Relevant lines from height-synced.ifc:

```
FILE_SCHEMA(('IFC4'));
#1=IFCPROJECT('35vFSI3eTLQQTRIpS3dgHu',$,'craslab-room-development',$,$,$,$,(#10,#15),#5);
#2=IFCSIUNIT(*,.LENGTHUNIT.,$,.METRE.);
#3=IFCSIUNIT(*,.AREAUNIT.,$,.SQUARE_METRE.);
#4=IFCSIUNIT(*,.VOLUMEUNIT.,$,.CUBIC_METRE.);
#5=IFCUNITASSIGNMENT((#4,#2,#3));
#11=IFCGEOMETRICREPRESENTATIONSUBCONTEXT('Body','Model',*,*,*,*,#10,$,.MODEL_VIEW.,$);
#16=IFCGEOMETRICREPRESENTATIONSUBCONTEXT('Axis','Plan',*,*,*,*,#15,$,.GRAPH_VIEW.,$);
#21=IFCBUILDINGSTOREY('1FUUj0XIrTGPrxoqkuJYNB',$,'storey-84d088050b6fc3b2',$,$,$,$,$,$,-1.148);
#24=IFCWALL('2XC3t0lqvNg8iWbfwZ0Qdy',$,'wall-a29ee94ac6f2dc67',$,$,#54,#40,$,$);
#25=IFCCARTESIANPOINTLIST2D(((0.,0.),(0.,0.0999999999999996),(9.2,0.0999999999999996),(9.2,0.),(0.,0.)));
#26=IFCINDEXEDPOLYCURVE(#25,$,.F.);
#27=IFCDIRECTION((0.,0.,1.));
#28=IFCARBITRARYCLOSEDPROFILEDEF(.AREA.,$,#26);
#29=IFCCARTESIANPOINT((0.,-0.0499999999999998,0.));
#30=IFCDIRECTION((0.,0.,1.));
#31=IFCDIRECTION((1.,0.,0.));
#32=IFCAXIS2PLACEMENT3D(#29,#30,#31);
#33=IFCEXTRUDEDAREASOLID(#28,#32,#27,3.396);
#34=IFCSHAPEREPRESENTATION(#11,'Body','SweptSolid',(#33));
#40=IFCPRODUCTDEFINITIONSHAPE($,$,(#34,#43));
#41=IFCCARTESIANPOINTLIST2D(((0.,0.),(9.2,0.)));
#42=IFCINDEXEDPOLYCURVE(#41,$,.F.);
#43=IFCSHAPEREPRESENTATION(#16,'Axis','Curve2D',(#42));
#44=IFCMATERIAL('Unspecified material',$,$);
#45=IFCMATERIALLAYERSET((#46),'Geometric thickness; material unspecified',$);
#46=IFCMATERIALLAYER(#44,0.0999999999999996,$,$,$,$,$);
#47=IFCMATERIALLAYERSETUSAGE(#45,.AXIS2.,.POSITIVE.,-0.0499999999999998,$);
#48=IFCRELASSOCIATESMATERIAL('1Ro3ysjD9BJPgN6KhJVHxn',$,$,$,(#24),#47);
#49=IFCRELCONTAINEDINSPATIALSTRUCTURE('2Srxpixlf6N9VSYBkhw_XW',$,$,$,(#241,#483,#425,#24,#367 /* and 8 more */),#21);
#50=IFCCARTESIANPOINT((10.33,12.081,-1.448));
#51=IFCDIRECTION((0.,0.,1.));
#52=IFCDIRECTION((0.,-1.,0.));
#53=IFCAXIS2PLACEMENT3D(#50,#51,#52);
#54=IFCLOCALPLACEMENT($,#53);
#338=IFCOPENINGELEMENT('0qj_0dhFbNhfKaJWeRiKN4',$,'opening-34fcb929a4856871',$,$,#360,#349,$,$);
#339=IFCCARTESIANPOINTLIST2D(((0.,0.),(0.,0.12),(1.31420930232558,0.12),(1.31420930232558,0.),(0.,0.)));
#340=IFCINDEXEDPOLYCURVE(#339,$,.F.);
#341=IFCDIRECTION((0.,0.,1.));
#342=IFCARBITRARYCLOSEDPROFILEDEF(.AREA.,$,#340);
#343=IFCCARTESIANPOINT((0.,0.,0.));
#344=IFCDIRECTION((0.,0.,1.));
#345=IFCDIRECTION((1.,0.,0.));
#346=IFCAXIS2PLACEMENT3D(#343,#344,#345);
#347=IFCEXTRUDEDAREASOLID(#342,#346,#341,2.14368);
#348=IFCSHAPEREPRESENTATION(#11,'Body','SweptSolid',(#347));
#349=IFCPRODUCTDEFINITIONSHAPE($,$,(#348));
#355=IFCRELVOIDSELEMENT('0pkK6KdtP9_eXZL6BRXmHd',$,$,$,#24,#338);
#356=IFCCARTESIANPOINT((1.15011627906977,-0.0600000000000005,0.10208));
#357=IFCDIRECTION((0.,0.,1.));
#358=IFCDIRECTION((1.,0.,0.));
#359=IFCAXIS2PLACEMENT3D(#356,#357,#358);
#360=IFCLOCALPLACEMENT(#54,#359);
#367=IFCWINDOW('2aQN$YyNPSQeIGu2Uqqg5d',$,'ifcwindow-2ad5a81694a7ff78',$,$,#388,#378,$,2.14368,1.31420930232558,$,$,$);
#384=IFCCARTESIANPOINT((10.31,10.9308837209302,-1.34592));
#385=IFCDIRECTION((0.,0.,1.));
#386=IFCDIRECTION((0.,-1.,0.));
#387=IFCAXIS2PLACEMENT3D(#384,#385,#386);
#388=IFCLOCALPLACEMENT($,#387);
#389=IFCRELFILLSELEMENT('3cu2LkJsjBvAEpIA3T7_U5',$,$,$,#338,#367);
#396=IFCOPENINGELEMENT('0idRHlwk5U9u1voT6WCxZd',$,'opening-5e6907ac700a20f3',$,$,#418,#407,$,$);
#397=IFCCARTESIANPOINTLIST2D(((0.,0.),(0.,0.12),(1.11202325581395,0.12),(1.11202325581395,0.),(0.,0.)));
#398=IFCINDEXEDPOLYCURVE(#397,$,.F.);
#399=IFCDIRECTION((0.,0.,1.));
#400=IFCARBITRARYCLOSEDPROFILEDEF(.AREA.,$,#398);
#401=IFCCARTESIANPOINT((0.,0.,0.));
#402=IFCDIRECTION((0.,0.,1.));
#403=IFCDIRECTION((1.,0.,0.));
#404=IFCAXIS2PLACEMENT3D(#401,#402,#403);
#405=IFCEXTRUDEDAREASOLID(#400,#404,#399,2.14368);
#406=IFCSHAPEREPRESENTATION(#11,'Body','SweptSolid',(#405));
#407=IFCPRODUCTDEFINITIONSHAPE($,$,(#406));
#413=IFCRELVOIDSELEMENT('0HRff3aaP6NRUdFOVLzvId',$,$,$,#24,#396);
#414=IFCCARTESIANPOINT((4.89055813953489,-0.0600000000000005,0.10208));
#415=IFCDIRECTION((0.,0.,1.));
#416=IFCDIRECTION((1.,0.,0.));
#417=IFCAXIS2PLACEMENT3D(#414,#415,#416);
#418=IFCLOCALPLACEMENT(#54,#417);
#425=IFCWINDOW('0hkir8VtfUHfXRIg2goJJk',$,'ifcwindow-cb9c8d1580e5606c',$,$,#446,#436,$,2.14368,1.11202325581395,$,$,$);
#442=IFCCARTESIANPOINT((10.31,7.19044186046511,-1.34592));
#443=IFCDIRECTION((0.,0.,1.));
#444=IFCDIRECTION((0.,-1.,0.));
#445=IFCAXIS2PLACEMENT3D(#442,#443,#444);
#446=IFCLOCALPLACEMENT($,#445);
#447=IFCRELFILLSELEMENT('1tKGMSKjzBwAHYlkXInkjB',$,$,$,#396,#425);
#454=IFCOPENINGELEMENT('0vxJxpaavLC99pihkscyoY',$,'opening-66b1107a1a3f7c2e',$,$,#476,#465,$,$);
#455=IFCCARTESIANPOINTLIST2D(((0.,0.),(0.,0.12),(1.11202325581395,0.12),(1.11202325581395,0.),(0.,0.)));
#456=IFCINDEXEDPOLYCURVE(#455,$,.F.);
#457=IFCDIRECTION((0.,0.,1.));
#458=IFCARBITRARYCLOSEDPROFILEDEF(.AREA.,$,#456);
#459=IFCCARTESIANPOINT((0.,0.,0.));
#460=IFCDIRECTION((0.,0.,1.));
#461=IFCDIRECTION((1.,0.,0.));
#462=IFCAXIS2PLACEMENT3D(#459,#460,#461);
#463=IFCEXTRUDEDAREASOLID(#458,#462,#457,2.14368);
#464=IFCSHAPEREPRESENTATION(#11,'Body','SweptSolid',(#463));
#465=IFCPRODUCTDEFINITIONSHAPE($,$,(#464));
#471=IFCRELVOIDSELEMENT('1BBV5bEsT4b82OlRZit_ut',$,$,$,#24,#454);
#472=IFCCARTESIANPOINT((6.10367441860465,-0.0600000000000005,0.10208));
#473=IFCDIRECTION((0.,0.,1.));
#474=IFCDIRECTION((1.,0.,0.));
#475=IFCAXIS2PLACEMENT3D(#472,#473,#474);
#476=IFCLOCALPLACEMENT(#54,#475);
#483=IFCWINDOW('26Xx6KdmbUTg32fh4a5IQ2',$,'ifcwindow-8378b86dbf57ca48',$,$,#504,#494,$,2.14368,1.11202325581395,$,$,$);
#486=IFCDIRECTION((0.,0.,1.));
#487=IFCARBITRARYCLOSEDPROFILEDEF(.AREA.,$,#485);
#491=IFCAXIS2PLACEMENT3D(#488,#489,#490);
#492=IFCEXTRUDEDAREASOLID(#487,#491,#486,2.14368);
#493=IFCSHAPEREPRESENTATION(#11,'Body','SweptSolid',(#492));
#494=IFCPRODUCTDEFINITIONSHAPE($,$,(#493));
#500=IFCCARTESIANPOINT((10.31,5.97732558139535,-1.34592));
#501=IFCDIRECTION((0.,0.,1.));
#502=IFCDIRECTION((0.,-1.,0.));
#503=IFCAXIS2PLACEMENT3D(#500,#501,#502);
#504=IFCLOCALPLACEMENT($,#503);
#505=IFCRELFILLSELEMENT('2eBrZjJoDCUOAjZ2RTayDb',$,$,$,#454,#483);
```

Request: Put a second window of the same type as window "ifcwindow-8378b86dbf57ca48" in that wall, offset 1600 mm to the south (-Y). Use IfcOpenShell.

```python
import ifcopenshell
import ifcopenshell.api.feature
import ifcopenshell.api.geometry
import ifcopenshell.api.root
import ifcopenshell.geom
import ifcopenshell.util.element
import ifcopenshell.util.placement
import ifcopenshell.util.shape
import ifcopenshell.util.unit

model = ifcopenshell.open("height-synced.ifc")
unit_scale = ifcopenshell.util.unit.calculate_unit_scale(model)
settings = ifcopenshell.geom.settings()


def volume(element):
    """Net volume in cubic metres, openings subtracted."""
    shape = ifcopenshell.geom.create_shape(settings, element)
    return ifcopenshell.util.shape.get_volume(shape.geometry)


window = model.by_guid("26Xx6KdmbUTg32fh4a5IQ2")
opening = window.FillsVoids[0].RelatingOpeningElement
wall = opening.VoidsElements[0].RelatingBuildingElement
before = volume(wall)
shift = ifcopenshell.util.placement.get_local_placement(wall.ObjectPlacement)[:3, 0] * 1.6 / unit_scale

# copy_class copies the void relationship, type, container and properties, but no geometry.
new_opening = ifcopenshell.api.root.copy_class(model, product=opening)
new_opening.Representation = ifcopenshell.util.element.copy_deep(
    model, opening.Representation, exclude=["IfcGeometricRepresentationContext", "IfcRepresentationMap"]
)
new_window = ifcopenshell.api.root.copy_class(model, product=window)
new_window.Representation = ifcopenshell.util.element.copy_deep(
    model, window.Representation, exclude=["IfcGeometricRepresentationContext", "IfcRepresentationMap"]
)
ifcopenshell.api.feature.add_filling(model, opening=new_opening, element=new_window)

for old, new in ((opening, new_opening), (window, new_window)):
    matrix = ifcopenshell.util.placement.get_local_placement(old.ObjectPlacement)
    matrix[:3, 3] += shift
    ifcopenshell.api.geometry.edit_object_placement(model, product=new, matrix=matrix, is_si=False)

after = volume(wall)

print(f"wall volume {before:.3f} -> {after:.3f} m3")

model.write("height-synced_edited.ifc")
```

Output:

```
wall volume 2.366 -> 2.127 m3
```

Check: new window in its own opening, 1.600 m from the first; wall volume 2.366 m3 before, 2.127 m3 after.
